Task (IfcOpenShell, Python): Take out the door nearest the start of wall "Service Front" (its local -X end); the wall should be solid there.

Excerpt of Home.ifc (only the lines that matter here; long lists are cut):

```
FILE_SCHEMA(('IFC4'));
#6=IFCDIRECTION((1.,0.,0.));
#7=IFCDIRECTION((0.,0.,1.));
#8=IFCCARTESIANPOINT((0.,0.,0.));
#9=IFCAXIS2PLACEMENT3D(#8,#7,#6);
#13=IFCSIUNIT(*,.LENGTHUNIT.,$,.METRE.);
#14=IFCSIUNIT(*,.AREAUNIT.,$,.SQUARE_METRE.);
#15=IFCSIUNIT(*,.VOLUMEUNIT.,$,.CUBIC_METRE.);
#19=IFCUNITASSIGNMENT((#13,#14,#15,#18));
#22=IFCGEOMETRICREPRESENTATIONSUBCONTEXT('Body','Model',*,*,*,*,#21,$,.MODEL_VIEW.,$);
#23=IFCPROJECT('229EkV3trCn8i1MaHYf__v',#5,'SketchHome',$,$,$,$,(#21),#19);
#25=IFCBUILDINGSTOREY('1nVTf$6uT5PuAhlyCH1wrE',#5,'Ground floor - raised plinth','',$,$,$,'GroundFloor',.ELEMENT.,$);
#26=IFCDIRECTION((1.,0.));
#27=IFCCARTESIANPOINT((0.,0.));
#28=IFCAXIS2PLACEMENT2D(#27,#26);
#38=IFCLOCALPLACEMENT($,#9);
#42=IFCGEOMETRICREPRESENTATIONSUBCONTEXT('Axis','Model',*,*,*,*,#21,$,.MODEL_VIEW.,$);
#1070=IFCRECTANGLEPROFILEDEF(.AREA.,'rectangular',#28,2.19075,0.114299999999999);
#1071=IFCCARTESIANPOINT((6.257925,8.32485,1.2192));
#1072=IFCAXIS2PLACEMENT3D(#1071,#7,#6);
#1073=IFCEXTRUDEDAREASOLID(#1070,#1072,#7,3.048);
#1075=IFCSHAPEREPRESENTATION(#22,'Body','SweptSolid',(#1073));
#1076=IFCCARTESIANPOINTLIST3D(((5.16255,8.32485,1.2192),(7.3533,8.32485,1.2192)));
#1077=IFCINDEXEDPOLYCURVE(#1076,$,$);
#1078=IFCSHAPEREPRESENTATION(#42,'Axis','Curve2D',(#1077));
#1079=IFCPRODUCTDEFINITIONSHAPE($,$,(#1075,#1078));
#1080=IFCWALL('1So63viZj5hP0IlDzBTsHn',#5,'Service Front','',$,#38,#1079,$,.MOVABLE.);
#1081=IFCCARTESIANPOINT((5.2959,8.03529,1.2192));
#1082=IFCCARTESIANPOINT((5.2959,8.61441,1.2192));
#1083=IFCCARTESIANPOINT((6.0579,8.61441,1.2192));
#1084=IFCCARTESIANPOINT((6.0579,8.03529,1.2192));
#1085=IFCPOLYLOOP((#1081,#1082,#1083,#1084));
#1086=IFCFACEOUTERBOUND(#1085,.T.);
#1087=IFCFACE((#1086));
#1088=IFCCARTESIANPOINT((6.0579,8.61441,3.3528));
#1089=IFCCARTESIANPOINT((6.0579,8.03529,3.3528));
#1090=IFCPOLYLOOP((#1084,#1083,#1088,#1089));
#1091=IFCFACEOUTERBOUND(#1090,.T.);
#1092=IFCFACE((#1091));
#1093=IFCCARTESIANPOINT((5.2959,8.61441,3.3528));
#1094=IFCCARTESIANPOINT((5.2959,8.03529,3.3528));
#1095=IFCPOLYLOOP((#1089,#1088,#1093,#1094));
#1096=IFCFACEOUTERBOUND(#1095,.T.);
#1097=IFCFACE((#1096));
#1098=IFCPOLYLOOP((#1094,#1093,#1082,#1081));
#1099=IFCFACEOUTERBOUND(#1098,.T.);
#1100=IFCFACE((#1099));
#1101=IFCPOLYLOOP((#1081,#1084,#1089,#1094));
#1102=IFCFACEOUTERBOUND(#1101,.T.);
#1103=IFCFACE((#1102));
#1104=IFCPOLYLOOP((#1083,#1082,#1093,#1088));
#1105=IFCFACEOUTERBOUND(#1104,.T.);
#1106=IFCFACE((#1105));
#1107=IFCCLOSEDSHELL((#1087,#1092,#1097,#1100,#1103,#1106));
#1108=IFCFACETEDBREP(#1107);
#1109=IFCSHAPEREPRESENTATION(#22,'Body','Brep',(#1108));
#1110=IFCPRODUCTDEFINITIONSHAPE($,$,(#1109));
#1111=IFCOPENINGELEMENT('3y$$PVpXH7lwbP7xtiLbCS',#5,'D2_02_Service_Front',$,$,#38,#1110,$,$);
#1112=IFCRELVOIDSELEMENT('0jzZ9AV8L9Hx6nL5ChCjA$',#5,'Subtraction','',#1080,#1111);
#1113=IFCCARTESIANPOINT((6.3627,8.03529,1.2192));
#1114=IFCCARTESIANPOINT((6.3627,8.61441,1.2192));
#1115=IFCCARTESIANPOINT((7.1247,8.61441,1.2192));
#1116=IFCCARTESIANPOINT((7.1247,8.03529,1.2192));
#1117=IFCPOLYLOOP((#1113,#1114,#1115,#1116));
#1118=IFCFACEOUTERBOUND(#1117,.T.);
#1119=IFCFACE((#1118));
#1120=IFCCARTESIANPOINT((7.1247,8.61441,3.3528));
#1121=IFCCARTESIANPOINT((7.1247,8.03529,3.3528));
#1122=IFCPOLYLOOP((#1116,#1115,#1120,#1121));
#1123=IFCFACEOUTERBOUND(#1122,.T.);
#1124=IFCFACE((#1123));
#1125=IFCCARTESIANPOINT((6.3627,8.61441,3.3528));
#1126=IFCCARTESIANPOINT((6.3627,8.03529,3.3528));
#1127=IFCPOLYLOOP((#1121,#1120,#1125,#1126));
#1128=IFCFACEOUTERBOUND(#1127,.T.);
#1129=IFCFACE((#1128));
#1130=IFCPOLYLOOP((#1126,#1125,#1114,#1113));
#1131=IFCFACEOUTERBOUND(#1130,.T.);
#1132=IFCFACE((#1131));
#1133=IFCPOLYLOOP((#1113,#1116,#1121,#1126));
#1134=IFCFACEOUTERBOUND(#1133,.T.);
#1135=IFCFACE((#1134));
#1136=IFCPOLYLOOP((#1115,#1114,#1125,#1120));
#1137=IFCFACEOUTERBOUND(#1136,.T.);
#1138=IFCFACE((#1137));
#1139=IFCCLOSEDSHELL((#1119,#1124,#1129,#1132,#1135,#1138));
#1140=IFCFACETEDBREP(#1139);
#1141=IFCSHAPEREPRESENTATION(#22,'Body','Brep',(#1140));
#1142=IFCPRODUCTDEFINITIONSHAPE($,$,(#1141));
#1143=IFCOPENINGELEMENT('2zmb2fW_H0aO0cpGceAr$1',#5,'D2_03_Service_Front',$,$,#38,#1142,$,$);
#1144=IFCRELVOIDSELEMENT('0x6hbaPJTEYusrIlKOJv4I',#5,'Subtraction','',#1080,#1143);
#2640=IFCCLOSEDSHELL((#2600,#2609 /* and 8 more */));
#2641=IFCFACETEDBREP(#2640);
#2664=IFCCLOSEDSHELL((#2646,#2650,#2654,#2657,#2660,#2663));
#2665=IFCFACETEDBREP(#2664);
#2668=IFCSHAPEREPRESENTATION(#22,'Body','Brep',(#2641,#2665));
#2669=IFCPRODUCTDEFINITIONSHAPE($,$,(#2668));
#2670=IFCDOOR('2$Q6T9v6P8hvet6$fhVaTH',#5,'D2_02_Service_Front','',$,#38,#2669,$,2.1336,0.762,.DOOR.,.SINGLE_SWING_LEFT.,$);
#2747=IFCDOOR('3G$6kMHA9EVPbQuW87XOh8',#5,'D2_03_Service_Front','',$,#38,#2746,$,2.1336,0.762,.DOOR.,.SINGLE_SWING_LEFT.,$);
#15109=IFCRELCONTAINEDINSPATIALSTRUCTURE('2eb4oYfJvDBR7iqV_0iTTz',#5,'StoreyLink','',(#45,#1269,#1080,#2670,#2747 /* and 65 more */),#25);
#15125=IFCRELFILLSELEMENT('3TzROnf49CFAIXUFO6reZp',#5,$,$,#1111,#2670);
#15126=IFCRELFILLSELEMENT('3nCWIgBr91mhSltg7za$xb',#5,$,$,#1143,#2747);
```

```python
import ifcopenshell
import ifcopenshell.api.feature
import ifcopenshell.api.root
import ifcopenshell.geom
import ifcopenshell.util.shape

model = ifcopenshell.open("Home.ifc")
settings = ifcopenshell.geom.settings()


def volume(element):
    """Net volume in cubic metres, openings subtracted."""
    shape = ifcopenshell.geom.create_shape(settings, element)
    return ifcopenshell.util.shape.get_volume(shape.geometry)


door = model.by_guid("2$Q6T9v6P8hvet6$fhVaTH")
opening = door.FillsVoids[0].RelatingOpeningElement
wall = opening.VoidsElements[0].RelatingBuildingElement
before = volume(wall)

ifcopenshell.api.root.remove_product(model, product=door)
ifcopenshell.api.feature.remove_feature(model, feature=opening)

after = volume(wall)

print(f"wall volume {before:.3f} -> {after:.3f} m3")

model.write("Home_updated.ifc")
```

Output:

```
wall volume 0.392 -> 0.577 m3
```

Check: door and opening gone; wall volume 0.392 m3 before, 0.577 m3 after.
